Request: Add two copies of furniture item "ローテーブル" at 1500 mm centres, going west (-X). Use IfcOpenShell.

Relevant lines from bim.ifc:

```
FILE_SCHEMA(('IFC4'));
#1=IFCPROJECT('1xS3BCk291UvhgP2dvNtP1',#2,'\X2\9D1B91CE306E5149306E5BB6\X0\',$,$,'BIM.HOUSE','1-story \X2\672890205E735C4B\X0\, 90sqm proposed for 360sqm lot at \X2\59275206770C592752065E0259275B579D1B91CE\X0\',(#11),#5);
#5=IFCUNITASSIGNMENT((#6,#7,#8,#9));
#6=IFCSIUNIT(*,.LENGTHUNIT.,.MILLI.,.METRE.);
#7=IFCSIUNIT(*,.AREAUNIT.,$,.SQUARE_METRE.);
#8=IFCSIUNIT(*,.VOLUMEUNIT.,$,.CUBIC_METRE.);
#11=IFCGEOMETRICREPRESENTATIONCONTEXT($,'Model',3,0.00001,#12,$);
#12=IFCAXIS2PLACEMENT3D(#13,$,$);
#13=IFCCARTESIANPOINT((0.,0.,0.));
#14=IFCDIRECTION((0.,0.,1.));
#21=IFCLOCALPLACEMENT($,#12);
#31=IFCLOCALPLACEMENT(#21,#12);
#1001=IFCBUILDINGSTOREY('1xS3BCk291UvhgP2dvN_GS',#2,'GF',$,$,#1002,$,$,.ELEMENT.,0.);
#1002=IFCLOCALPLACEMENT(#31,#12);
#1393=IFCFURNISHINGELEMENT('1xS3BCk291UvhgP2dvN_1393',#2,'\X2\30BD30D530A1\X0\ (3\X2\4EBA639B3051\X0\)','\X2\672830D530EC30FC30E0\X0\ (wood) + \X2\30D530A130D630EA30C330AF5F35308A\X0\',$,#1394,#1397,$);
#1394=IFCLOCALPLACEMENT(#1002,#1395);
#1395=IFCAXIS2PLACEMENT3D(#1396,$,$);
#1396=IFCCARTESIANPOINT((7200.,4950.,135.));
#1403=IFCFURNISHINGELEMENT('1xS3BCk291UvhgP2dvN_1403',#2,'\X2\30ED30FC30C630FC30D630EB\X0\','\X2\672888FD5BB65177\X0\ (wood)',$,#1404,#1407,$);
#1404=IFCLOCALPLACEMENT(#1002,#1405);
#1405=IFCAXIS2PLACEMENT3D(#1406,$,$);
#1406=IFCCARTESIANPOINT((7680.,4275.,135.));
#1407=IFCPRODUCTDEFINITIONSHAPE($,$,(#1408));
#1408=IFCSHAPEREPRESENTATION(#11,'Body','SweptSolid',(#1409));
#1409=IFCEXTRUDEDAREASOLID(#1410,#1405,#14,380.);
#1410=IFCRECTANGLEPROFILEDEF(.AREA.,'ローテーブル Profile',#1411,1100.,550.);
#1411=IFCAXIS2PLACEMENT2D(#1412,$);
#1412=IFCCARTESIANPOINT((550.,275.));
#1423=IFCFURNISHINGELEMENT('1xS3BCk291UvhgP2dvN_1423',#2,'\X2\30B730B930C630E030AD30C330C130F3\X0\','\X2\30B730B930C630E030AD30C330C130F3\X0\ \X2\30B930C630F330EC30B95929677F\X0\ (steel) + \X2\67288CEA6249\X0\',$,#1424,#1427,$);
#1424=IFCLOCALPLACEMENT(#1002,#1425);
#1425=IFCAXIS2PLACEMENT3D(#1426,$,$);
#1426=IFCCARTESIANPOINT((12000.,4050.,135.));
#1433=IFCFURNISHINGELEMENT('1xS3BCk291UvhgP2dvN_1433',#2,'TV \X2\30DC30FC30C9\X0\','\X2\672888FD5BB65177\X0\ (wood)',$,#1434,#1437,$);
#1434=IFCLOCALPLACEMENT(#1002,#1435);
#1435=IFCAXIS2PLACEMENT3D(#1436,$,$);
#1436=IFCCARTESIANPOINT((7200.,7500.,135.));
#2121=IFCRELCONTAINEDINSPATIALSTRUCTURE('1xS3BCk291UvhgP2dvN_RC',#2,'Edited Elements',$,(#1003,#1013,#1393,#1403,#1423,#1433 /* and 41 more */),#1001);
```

```python
import numpy as np
import ifcopenshell
import ifcopenshell.api.geometry
import ifcopenshell.api.root
import ifcopenshell.util.element
import ifcopenshell.util.placement
import ifcopenshell.util.unit

model = ifcopenshell.open("bim.ifc")
unit_scale = ifcopenshell.util.unit.calculate_unit_scale(model)


def reuse_history(source, copy):
    """copy_class also copies each property set's owner history, people and application; keep the originals."""
    for rel in copy.IsDefinedBy:
        if rel.is_a("IfcRelDefinesByProperties") and (history := rel.RelatingPropertyDefinition.OwnerHistory):
            rel.RelatingPropertyDefinition.OwnerHistory = source.OwnerHistory
            ifcopenshell.util.element.remove_deep2(model, history)


source = model.by_guid("1xS3BCk291UvhgP2dvN_1403")
base = ifcopenshell.util.placement.get_local_placement(source.ObjectPlacement)
step = np.array([-1.0, 0.0, 0.0]) * 1.5 / unit_scale

for i in range(1, 3):
    copy = ifcopenshell.api.root.copy_class(model, product=source)
    copy.Representation = ifcopenshell.util.element.copy_deep(
        model, source.Representation, exclude=["IfcGeometricRepresentationContext", "IfcRepresentationMap"]
    )
    reuse_history(source, copy)
    matrix = base.copy()
    matrix[:3, 3] += i * step
    print("added at", matrix[:3, 3].round(3) + 0.0)
    ifcopenshell.api.geometry.edit_object_placement(model, product=copy, matrix=matrix, is_si=False)

model.write("bim_edited.ifc")
```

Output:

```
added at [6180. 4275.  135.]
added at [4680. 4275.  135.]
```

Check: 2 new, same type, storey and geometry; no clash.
